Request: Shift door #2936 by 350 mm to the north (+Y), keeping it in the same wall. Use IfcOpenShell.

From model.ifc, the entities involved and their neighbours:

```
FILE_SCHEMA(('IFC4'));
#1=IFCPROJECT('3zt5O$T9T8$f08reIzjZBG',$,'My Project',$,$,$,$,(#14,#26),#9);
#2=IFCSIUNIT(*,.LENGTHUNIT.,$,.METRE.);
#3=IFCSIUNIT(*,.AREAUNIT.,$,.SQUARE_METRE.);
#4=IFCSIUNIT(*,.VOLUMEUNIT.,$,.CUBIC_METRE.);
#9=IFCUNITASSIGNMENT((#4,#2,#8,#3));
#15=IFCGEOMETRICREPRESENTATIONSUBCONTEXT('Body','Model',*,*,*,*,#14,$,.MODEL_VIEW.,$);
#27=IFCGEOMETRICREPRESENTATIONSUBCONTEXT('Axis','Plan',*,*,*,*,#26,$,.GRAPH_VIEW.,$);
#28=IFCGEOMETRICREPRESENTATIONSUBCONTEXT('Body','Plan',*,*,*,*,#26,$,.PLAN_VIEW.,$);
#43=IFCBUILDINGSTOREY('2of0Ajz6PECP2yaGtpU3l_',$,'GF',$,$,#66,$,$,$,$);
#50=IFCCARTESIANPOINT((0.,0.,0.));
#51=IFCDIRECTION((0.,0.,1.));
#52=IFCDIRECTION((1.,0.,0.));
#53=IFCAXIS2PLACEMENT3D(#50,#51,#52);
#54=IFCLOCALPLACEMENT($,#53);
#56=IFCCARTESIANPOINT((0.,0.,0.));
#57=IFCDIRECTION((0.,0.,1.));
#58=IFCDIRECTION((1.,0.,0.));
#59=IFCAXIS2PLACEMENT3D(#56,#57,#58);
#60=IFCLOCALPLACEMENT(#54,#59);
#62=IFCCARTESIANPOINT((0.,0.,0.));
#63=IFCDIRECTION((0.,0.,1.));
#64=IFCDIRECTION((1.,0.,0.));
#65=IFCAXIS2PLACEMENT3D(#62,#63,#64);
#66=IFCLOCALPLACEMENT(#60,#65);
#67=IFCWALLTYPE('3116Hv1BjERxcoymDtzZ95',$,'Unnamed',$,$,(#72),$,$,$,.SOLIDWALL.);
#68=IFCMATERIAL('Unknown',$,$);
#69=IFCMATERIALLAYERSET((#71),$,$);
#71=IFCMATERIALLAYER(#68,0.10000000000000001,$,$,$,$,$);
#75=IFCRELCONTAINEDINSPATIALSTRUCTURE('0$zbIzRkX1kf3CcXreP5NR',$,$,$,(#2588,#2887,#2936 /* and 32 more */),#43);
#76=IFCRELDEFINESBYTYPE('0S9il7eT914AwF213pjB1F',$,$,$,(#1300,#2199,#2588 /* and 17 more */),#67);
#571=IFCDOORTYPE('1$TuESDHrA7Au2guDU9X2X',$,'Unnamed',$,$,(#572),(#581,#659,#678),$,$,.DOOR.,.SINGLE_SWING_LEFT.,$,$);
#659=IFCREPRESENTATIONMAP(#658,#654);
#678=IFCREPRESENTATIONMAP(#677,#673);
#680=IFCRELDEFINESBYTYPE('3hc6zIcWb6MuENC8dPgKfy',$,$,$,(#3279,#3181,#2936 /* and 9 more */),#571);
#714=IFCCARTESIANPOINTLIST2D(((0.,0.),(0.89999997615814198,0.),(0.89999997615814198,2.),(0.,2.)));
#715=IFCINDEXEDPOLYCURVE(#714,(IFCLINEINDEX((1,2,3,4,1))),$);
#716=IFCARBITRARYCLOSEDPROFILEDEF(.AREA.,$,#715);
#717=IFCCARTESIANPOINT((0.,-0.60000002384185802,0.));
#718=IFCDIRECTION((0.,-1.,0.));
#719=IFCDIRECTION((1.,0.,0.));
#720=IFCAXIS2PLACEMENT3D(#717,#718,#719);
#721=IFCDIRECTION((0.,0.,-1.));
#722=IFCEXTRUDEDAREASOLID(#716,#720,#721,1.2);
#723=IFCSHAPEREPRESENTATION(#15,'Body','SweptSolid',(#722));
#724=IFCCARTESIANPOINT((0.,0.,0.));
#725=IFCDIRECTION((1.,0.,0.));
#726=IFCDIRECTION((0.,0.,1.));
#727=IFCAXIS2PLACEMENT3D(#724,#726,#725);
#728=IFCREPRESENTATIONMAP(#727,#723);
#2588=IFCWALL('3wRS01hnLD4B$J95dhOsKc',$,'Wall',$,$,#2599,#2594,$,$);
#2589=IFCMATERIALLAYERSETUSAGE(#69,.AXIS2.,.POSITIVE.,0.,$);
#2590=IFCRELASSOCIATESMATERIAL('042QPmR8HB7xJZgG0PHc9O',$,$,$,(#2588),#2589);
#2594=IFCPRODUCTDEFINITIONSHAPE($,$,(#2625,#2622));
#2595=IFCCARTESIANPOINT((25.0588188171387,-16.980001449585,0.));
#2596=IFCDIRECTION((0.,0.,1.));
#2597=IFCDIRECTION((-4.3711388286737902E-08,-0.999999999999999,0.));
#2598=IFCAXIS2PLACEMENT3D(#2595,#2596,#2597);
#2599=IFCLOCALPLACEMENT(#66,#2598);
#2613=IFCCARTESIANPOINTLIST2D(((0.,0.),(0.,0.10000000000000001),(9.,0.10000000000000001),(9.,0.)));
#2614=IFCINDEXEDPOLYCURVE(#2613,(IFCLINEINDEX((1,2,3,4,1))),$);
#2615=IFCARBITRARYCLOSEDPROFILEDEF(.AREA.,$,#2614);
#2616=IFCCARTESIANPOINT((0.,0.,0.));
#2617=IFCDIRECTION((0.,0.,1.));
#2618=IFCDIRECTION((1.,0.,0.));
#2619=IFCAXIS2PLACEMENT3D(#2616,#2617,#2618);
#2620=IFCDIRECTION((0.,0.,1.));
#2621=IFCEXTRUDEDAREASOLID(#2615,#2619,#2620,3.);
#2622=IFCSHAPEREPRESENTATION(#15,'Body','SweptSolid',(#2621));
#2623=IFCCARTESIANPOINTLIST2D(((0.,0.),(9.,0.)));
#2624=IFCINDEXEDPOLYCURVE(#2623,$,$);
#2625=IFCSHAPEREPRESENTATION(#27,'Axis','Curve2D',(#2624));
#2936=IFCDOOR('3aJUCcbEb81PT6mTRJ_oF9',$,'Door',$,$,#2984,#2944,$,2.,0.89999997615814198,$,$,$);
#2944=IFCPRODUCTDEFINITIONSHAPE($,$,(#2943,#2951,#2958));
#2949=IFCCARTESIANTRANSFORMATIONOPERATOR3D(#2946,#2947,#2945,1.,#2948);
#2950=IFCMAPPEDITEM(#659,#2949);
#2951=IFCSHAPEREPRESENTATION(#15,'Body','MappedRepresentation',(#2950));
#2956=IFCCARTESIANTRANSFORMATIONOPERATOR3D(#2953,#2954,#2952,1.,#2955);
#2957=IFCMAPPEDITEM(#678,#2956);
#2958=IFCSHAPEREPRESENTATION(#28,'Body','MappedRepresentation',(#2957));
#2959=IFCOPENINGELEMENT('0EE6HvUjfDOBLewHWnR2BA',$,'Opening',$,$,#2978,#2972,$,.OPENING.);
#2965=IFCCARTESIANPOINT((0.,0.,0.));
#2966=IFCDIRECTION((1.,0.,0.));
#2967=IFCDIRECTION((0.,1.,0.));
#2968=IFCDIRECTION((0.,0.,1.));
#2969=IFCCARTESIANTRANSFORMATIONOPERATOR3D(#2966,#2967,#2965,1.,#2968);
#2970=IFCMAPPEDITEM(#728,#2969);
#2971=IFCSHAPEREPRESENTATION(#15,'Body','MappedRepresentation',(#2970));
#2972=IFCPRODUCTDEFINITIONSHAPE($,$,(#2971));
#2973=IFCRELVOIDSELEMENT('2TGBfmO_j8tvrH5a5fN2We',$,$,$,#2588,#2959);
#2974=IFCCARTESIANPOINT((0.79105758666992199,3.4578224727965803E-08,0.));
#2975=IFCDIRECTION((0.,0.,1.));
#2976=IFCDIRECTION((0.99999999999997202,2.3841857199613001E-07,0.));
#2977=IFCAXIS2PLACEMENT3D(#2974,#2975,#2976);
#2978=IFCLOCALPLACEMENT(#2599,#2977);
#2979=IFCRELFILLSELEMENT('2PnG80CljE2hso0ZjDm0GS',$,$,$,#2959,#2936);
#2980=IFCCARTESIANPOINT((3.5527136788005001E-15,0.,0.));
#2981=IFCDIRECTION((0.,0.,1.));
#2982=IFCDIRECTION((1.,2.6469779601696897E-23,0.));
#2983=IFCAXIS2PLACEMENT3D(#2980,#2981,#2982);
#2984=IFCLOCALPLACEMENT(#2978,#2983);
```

```python
import ifcopenshell
import ifcopenshell.api.geometry
import ifcopenshell.util.placement
import ifcopenshell.util.unit

model = ifcopenshell.open("model.ifc")
unit_scale = ifcopenshell.util.unit.calculate_unit_scale(model)

door = model.by_id(2936)
opening = door.FillsVoids[0].RelatingOpeningElement
wall = opening.VoidsElements[0].RelatingBuildingElement

wall_matrix = ifcopenshell.util.placement.get_local_placement(wall.ObjectPlacement)
shift = wall_matrix[:3, 0] * -0.35 / unit_scale
before = ifcopenshell.util.placement.get_local_placement(door.ObjectPlacement)[:3, 3].copy()

# The door is placed relative to its opening, so it follows when the opening moves.
matrix = ifcopenshell.util.placement.get_local_placement(opening.ObjectPlacement)
matrix[:3, 3] += shift
ifcopenshell.api.geometry.edit_object_placement(
    model, product=opening, matrix=matrix, is_si=False, should_transform_children=True
)

after = ifcopenshell.util.placement.get_local_placement(door.ObjectPlacement)[:3, 3]
print("door moved by", (after - before).round(3) + 0.0)

model.write("model_edited.ifc")
```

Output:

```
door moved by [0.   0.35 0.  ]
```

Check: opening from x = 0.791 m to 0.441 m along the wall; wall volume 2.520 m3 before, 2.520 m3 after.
